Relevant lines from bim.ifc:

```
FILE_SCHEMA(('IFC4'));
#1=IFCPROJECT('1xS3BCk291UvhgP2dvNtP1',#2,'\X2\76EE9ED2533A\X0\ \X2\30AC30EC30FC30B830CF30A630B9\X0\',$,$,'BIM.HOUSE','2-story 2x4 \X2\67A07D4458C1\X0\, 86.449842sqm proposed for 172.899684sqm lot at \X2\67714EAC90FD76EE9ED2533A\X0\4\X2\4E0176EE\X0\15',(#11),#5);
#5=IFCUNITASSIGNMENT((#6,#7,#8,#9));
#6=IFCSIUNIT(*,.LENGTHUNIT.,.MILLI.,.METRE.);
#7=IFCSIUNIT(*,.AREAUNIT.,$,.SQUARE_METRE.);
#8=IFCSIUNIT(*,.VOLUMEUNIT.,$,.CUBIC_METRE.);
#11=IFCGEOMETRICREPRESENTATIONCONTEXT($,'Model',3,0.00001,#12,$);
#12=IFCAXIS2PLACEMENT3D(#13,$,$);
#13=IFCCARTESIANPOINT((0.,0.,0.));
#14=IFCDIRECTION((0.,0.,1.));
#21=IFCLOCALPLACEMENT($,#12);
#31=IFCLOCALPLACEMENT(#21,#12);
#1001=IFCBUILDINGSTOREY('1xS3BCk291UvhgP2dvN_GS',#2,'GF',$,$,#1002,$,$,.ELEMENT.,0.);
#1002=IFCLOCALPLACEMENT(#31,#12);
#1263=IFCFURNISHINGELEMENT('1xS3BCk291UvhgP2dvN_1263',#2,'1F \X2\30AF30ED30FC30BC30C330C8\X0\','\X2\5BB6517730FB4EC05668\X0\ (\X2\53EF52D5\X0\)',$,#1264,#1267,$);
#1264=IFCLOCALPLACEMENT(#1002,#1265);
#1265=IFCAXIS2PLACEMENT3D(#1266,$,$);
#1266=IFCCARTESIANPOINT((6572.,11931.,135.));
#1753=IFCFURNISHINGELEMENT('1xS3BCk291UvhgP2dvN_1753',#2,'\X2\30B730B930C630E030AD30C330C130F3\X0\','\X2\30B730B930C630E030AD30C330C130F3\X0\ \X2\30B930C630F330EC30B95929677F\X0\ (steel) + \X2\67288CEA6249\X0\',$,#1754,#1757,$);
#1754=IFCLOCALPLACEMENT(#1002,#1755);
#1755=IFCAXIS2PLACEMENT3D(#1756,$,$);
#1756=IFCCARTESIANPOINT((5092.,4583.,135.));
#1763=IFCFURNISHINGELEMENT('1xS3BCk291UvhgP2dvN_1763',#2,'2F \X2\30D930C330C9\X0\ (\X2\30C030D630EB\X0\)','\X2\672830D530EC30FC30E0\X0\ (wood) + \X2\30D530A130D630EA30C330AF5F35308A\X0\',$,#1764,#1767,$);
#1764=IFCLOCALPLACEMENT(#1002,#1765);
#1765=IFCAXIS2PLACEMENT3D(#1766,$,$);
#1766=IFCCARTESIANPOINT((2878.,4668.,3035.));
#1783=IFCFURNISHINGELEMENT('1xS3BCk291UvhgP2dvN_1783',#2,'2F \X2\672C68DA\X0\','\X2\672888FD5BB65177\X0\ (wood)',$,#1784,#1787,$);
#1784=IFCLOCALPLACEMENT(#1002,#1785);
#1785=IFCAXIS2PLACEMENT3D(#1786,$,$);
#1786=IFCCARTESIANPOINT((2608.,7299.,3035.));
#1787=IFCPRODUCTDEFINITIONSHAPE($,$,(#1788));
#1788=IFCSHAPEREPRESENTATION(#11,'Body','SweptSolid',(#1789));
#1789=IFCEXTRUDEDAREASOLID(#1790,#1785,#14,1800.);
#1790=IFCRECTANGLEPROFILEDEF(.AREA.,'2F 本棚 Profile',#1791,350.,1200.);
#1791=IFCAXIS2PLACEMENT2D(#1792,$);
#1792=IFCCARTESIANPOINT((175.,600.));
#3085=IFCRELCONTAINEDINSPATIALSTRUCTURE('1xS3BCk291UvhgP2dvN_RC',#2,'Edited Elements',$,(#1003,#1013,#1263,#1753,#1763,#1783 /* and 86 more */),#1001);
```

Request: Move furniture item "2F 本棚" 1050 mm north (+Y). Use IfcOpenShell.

```python
import ifcopenshell
import ifcopenshell.api.geometry
import ifcopenshell.util.placement

model = ifcopenshell.open("bim.ifc")

item = model.by_guid("1xS3BCk291UvhgP2dvN_1783")
matrix = ifcopenshell.util.placement.get_local_placement(item.ObjectPlacement)
matrix[1, 3] += 1050.0
ifcopenshell.api.geometry.edit_object_placement(model, product=item, matrix=matrix, is_si=False)

print(ifcopenshell.util.placement.get_local_placement(item.ObjectPlacement).round(3) + 0.0)

model.write("bim-out.ifc")
```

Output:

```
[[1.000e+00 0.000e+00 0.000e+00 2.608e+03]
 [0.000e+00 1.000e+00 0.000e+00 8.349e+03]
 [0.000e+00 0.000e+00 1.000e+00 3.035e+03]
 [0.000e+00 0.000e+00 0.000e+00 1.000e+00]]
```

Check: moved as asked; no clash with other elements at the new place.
